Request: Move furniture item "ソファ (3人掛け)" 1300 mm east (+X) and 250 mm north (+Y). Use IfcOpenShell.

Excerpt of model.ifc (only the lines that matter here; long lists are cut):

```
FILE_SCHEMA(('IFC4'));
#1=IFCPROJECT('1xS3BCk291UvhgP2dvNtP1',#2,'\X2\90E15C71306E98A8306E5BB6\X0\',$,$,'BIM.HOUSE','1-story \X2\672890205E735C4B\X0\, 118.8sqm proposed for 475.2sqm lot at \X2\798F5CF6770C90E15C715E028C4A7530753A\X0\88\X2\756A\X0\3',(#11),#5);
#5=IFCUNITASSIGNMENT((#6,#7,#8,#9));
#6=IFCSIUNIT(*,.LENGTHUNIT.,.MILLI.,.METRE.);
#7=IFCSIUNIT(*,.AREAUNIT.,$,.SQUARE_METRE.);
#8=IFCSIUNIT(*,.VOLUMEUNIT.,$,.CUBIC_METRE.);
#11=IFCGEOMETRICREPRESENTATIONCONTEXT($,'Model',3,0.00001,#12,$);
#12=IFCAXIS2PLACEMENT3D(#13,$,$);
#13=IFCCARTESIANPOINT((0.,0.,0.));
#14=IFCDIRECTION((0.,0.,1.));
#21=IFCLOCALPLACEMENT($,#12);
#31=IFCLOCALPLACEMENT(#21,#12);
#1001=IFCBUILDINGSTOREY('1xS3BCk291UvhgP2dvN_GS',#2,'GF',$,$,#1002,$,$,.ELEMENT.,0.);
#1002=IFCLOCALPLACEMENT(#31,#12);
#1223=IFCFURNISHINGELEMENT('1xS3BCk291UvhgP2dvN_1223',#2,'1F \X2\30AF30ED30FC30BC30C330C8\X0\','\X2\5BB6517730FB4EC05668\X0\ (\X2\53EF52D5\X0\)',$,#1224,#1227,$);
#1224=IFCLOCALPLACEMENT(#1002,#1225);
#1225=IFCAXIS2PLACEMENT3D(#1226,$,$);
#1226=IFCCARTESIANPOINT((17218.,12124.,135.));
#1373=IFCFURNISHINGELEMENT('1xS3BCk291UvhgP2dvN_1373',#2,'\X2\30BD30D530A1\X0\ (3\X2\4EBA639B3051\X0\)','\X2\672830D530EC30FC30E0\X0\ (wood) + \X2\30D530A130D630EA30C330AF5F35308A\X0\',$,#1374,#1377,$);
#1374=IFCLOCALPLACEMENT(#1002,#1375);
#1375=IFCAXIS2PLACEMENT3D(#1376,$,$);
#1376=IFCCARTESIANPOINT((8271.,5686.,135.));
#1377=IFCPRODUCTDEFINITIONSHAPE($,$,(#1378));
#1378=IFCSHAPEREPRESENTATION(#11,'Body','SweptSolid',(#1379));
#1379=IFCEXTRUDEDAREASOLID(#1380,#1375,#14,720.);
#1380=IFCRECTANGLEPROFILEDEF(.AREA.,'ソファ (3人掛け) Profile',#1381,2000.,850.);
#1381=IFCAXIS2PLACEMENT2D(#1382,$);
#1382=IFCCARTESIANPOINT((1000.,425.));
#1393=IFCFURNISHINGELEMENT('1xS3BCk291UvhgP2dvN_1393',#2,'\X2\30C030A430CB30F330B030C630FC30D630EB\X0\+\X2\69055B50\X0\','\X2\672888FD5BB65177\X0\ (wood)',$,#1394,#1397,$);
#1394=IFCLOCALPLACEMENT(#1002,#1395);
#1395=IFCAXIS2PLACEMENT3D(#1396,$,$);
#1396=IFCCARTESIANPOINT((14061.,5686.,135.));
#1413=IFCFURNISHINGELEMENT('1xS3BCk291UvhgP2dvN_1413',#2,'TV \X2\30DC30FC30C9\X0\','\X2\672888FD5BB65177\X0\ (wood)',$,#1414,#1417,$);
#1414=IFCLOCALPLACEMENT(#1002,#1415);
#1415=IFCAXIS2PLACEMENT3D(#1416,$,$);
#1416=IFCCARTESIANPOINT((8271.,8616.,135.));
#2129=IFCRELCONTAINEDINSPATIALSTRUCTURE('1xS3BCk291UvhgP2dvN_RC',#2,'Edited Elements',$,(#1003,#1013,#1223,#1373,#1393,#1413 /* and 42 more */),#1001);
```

```python
import ifcopenshell
import ifcopenshell.api.geometry
import ifcopenshell.util.placement
import ifcopenshell.util.unit

model = ifcopenshell.open("model.ifc")
unit_scale = ifcopenshell.util.unit.calculate_unit_scale(model)

item = model.by_id(1373)
matrix = ifcopenshell.util.placement.get_local_placement(item.ObjectPlacement)
matrix[0, 3] += 1.3 / unit_scale
matrix[1, 3] += 0.25 / unit_scale
ifcopenshell.api.geometry.edit_object_placement(model, product=item, matrix=matrix, is_si=False)

print(ifcopenshell.util.placement.get_local_placement(item.ObjectPlacement).round(3) + 0.0)

model.write("model_v2.ifc")
```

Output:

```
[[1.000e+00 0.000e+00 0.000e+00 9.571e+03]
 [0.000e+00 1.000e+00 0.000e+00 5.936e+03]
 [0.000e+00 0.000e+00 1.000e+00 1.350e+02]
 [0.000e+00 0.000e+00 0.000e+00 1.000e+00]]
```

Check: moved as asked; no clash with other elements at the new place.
